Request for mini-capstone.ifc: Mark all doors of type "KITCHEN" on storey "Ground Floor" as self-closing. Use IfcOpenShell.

First a look at what the model holds.

```python
import ifcopenshell
import ifcopenshell.util.element

model = ifcopenshell.open("mini-capstone.ifc")
print(model.schema)
storey = next(s for s in model.by_type("IfcBuildingStorey") if s.Name == "Ground Floor")
doors = [e for e in ifcopenshell.util.element.get_decomposition(storey) if e.is_a("IfcDoor")]
seen = {}
for e in doors:
    element_type = ifcopenshell.util.element.get_type(e)
    key = (element_type.Name if element_type != e and element_type else None, ifcopenshell.util.element.get_pset(e, "Pset_DoorCommon", "SelfClosing"))
    seen[key] = seen.get(key, 0) + 1
for (name, value), count in sorted(seen.items(), key=str):
    print(count, "x", name, "|", value)
```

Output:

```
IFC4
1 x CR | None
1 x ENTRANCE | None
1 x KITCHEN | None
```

```python
import ifcopenshell
import ifcopenshell.api.pset
import ifcopenshell.util.element

model = ifcopenshell.open("mini-capstone.ifc")

storey = next(s for s in model.by_type("IfcBuildingStorey") if s.Name == "Ground Floor")
doors = [e for e in ifcopenshell.util.element.get_decomposition(storey) if e.is_a("IfcDoor")]

count = 0
for e in doors:
    element_type = ifcopenshell.util.element.get_type(e)
    if element_type in (None, e) or element_type.Name != "KITCHEN":
        continue
    # add_pset returns the element's existing set when there is one.
    pset = ifcopenshell.api.pset.add_pset(model, product=e, name="Pset_DoorCommon")
    ifcopenshell.api.pset.edit_pset(model, pset=pset, properties={"SelfClosing": True})
    count += 1

print(count, "doors updated")

model.write("mini-capstone-out.ifc")
```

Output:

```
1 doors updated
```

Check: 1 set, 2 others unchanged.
